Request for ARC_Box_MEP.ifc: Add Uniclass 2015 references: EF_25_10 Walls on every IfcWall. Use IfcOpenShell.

First a look at what the model holds.

```python
import ifcopenshell

model = ifcopenshell.open("ARC_Box_MEP.ifc")
print(model.schema)
print("classifications:", [c.Name for c in model.by_type("IfcClassification")])
for ifc_class in ("IfcDoor", "IfcRoof", "IfcStair", "IfcWall", "IfcWindow"):
    print(ifc_class, len(model.by_type(ifc_class)))
```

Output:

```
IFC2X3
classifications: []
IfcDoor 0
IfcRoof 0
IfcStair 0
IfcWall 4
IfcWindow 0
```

```python
import ifcopenshell
import ifcopenshell.api.classification

model = ifcopenshell.open("ARC_Box_MEP.ifc")

# IFC2X3 requires Source and Edition and has no link from the project to the system.
system = model.create_entity("IfcClassification", Source="NBS", Edition="2015", Name="Uniclass 2015")

codes = {
    "IfcWall": ("EF_25_10", "Walls"),
}
for ifc_class, (code, name) in codes.items():
    products = model.by_type(ifc_class)
    ifcopenshell.api.classification.add_reference(
        model, products=products, classification=system, identification=code, name=name
    )
    print(code, len(products))

model.write("ARC_Box_MEP_edited.ifc")
```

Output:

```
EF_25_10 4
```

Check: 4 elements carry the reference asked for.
